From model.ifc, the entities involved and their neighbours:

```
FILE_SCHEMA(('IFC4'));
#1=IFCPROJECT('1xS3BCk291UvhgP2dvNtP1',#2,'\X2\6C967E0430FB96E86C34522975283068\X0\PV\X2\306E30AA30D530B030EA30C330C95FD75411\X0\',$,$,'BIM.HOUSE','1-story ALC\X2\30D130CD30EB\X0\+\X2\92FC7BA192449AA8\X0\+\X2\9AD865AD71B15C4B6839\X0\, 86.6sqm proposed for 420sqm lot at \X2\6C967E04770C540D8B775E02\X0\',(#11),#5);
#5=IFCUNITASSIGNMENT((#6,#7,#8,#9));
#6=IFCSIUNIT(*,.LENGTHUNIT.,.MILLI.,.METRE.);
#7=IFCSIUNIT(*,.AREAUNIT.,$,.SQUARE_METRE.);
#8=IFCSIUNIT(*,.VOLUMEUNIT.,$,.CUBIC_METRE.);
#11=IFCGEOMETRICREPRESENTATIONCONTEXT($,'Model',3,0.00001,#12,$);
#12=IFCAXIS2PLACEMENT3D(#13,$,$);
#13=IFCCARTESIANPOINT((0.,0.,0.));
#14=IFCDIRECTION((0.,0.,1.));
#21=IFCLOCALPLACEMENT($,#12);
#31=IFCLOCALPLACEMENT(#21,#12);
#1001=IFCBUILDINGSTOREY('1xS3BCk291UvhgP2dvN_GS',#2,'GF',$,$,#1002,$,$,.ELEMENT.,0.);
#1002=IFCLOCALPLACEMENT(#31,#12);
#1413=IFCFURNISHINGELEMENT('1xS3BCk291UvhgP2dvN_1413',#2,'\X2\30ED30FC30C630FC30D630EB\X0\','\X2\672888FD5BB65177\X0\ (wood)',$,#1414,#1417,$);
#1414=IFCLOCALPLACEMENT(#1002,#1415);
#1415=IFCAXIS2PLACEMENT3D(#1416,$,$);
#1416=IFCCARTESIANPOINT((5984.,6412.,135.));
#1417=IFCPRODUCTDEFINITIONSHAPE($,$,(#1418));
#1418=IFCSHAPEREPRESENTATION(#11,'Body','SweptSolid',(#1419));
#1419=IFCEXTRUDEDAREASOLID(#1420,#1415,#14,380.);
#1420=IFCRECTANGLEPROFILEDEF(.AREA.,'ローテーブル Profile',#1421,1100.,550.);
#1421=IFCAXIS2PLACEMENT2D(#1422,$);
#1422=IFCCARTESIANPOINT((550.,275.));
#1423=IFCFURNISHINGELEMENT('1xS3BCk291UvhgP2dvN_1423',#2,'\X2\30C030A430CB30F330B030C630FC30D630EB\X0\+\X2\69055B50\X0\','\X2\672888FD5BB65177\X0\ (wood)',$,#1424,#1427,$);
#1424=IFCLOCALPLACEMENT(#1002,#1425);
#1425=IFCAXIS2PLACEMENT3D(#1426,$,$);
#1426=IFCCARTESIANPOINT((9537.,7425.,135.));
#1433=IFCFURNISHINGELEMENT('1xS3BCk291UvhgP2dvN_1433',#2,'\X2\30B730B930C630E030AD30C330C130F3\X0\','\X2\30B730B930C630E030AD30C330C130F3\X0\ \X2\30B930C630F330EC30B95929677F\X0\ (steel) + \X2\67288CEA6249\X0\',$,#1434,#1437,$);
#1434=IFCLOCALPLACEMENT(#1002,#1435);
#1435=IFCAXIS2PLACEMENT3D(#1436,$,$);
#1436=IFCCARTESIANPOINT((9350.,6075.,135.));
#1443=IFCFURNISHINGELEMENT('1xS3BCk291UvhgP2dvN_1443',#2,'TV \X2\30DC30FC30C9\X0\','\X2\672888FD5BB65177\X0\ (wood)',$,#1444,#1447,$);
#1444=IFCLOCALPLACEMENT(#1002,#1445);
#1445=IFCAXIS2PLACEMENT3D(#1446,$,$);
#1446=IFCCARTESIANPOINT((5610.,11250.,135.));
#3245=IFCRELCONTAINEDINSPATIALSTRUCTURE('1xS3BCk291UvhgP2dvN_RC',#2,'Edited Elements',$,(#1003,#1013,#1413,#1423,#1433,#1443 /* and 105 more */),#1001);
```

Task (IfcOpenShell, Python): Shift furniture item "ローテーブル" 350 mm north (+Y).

```python
import ifcopenshell
import ifcopenshell.api.geometry
import ifcopenshell.util.placement
import ifcopenshell.util.unit

model = ifcopenshell.open("model.ifc")
unit_scale = ifcopenshell.util.unit.calculate_unit_scale(model)

item = model.by_guid("1xS3BCk291UvhgP2dvN_1413")
matrix = ifcopenshell.util.placement.get_local_placement(item.ObjectPlacement)
matrix[1, 3] += 0.35 / unit_scale
ifcopenshell.api.geometry.edit_object_placement(model, product=item, matrix=matrix, is_si=False)

print(ifcopenshell.util.placement.get_local_placement(item.ObjectPlacement).round(3) + 0.0)

model.write("model_edited.ifc")
```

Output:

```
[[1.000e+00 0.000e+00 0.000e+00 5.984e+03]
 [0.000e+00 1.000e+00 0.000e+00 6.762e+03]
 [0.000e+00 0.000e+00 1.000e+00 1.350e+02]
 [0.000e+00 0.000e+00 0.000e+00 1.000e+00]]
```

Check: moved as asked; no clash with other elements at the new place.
